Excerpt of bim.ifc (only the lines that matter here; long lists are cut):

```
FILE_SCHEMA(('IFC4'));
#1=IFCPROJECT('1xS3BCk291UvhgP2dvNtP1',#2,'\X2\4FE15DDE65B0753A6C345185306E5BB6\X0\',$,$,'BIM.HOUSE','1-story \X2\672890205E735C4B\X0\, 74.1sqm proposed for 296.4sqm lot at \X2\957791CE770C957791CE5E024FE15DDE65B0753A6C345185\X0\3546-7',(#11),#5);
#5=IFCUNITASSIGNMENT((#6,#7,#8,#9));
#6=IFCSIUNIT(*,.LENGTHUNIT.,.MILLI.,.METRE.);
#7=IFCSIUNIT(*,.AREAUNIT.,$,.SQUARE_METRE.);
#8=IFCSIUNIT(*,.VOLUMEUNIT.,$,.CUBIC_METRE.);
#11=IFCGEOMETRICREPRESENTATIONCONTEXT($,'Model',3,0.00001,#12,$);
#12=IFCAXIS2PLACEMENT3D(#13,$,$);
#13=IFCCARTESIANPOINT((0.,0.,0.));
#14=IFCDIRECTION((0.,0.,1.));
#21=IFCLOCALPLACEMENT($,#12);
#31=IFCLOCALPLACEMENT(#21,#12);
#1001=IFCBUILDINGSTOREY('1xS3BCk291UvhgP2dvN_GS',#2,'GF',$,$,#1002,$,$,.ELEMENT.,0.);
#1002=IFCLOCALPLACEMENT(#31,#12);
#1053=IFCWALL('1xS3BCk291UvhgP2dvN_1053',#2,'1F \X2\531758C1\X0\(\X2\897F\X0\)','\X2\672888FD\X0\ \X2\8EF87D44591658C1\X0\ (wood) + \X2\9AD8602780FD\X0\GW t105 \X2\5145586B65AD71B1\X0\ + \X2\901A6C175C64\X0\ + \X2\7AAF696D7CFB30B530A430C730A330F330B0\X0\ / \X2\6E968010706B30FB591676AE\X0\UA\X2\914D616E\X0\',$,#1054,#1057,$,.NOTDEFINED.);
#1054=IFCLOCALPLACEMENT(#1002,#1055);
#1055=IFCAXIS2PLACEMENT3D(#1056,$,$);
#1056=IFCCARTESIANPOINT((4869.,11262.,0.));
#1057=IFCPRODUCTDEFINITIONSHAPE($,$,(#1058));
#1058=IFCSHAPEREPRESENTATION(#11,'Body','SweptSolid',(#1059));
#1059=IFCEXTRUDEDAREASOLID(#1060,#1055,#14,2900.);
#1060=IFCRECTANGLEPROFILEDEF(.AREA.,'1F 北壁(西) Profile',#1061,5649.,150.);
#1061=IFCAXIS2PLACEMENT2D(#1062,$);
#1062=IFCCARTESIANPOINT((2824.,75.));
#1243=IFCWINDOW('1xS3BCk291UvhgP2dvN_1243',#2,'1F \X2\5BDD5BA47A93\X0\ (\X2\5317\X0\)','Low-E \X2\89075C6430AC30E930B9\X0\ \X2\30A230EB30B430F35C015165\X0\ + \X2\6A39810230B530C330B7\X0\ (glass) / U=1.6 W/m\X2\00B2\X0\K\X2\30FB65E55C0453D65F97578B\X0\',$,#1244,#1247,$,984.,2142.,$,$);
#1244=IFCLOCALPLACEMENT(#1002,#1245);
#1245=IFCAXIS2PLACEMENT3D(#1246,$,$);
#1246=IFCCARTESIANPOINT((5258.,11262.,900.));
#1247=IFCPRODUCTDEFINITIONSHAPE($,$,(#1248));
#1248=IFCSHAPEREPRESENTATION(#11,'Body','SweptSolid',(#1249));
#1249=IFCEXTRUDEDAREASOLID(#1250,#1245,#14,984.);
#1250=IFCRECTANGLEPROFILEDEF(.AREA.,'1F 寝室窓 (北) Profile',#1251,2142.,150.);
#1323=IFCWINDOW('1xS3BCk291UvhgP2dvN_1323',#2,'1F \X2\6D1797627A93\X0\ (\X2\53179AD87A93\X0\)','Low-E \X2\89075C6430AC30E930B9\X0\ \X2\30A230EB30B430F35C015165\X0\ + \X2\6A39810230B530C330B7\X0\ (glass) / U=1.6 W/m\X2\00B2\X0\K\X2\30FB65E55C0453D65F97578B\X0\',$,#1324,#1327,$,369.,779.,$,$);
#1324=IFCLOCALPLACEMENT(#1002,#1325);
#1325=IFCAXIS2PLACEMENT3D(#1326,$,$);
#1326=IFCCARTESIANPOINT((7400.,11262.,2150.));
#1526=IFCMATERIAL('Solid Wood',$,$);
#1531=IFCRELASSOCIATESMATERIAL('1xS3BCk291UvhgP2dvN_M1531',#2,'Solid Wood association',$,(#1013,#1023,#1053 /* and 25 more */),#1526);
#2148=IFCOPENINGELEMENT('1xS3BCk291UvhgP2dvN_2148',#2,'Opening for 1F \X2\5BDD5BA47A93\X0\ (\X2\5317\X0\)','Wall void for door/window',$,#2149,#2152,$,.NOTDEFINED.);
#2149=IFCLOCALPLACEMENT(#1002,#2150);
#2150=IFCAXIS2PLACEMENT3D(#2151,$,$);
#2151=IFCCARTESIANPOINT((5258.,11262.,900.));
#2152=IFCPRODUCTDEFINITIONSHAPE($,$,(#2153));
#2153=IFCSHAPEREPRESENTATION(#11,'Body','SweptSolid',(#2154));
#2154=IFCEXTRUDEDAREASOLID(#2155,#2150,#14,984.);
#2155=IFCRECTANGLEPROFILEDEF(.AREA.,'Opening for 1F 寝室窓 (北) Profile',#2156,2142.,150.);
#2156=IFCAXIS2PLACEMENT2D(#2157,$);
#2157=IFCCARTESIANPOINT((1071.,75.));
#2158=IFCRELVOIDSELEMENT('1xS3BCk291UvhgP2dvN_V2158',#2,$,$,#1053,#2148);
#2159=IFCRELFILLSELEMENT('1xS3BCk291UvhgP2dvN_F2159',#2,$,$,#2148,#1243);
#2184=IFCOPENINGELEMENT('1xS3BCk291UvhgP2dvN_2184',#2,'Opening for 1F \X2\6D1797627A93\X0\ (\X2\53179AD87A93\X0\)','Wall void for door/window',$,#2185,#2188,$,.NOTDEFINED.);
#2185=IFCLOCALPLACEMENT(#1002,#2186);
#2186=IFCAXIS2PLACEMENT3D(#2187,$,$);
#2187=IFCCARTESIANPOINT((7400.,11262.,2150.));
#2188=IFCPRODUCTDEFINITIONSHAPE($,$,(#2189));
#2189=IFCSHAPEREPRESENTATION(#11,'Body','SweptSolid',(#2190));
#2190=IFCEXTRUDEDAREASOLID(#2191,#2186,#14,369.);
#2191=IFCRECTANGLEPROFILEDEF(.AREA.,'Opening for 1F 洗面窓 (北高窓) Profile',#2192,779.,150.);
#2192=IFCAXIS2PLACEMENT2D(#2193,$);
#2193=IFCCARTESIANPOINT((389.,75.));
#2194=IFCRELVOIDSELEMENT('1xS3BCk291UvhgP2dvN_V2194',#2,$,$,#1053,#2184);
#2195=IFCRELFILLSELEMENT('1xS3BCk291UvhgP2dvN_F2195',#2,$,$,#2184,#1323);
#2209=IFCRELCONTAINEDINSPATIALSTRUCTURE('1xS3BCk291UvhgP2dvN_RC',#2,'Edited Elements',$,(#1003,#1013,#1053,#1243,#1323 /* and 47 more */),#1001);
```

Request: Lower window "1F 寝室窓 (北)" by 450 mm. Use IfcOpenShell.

```python
import numpy as np
import ifcopenshell
import ifcopenshell.api.geometry
import ifcopenshell.util.placement
import ifcopenshell.util.unit

model = ifcopenshell.open("bim.ifc")
unit_scale = ifcopenshell.util.unit.calculate_unit_scale(model)

window = model.by_id(1243)
opening = window.FillsVoids[0].RelatingOpeningElement
dz = -0.45 / unit_scale

shift = np.array([0.0, 0.0, dz])
# The window is not placed relative to its opening, so move both.
for product in (opening, window):
    matrix = ifcopenshell.util.placement.get_local_placement(product.ObjectPlacement)
    matrix[:3, 3] += shift
    ifcopenshell.api.geometry.edit_object_placement(model, product=product, matrix=matrix, is_si=False)

print(f"moved by {dz * unit_scale:+.3f} m")

model.write("bim_v2.ifc")
```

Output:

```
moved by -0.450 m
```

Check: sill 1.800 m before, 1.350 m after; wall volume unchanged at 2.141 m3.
